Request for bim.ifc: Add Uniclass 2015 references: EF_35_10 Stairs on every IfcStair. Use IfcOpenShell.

First a look at what the model holds.

```python
import ifcopenshell

model = ifcopenshell.open("bim.ifc")
print(model.schema)
print("classifications:", [c.Name for c in model.by_type("IfcClassification")])
for ifc_class in ("IfcDoor", "IfcRoof", "IfcStair", "IfcWall", "IfcWindow"):
    print(ifc_class, len(model.by_type(ifc_class)))
```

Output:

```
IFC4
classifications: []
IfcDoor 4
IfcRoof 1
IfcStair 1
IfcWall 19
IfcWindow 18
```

```python
import ifcopenshell
import ifcopenshell.api.classification

model = ifcopenshell.open("bim.ifc")

system = ifcopenshell.api.classification.add_classification(model, classification="Uniclass 2015")

codes = {
    "IfcStair": ("EF_35_10", "Stairs"),
}
for ifc_class, (code, name) in codes.items():
    products = model.by_type(ifc_class)
    ifcopenshell.api.classification.add_reference(
        model, products=products, classification=system, identification=code, name=name
    )
    print(code, len(products))

model.write("bim_rev.ifc")
```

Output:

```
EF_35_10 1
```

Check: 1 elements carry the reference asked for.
